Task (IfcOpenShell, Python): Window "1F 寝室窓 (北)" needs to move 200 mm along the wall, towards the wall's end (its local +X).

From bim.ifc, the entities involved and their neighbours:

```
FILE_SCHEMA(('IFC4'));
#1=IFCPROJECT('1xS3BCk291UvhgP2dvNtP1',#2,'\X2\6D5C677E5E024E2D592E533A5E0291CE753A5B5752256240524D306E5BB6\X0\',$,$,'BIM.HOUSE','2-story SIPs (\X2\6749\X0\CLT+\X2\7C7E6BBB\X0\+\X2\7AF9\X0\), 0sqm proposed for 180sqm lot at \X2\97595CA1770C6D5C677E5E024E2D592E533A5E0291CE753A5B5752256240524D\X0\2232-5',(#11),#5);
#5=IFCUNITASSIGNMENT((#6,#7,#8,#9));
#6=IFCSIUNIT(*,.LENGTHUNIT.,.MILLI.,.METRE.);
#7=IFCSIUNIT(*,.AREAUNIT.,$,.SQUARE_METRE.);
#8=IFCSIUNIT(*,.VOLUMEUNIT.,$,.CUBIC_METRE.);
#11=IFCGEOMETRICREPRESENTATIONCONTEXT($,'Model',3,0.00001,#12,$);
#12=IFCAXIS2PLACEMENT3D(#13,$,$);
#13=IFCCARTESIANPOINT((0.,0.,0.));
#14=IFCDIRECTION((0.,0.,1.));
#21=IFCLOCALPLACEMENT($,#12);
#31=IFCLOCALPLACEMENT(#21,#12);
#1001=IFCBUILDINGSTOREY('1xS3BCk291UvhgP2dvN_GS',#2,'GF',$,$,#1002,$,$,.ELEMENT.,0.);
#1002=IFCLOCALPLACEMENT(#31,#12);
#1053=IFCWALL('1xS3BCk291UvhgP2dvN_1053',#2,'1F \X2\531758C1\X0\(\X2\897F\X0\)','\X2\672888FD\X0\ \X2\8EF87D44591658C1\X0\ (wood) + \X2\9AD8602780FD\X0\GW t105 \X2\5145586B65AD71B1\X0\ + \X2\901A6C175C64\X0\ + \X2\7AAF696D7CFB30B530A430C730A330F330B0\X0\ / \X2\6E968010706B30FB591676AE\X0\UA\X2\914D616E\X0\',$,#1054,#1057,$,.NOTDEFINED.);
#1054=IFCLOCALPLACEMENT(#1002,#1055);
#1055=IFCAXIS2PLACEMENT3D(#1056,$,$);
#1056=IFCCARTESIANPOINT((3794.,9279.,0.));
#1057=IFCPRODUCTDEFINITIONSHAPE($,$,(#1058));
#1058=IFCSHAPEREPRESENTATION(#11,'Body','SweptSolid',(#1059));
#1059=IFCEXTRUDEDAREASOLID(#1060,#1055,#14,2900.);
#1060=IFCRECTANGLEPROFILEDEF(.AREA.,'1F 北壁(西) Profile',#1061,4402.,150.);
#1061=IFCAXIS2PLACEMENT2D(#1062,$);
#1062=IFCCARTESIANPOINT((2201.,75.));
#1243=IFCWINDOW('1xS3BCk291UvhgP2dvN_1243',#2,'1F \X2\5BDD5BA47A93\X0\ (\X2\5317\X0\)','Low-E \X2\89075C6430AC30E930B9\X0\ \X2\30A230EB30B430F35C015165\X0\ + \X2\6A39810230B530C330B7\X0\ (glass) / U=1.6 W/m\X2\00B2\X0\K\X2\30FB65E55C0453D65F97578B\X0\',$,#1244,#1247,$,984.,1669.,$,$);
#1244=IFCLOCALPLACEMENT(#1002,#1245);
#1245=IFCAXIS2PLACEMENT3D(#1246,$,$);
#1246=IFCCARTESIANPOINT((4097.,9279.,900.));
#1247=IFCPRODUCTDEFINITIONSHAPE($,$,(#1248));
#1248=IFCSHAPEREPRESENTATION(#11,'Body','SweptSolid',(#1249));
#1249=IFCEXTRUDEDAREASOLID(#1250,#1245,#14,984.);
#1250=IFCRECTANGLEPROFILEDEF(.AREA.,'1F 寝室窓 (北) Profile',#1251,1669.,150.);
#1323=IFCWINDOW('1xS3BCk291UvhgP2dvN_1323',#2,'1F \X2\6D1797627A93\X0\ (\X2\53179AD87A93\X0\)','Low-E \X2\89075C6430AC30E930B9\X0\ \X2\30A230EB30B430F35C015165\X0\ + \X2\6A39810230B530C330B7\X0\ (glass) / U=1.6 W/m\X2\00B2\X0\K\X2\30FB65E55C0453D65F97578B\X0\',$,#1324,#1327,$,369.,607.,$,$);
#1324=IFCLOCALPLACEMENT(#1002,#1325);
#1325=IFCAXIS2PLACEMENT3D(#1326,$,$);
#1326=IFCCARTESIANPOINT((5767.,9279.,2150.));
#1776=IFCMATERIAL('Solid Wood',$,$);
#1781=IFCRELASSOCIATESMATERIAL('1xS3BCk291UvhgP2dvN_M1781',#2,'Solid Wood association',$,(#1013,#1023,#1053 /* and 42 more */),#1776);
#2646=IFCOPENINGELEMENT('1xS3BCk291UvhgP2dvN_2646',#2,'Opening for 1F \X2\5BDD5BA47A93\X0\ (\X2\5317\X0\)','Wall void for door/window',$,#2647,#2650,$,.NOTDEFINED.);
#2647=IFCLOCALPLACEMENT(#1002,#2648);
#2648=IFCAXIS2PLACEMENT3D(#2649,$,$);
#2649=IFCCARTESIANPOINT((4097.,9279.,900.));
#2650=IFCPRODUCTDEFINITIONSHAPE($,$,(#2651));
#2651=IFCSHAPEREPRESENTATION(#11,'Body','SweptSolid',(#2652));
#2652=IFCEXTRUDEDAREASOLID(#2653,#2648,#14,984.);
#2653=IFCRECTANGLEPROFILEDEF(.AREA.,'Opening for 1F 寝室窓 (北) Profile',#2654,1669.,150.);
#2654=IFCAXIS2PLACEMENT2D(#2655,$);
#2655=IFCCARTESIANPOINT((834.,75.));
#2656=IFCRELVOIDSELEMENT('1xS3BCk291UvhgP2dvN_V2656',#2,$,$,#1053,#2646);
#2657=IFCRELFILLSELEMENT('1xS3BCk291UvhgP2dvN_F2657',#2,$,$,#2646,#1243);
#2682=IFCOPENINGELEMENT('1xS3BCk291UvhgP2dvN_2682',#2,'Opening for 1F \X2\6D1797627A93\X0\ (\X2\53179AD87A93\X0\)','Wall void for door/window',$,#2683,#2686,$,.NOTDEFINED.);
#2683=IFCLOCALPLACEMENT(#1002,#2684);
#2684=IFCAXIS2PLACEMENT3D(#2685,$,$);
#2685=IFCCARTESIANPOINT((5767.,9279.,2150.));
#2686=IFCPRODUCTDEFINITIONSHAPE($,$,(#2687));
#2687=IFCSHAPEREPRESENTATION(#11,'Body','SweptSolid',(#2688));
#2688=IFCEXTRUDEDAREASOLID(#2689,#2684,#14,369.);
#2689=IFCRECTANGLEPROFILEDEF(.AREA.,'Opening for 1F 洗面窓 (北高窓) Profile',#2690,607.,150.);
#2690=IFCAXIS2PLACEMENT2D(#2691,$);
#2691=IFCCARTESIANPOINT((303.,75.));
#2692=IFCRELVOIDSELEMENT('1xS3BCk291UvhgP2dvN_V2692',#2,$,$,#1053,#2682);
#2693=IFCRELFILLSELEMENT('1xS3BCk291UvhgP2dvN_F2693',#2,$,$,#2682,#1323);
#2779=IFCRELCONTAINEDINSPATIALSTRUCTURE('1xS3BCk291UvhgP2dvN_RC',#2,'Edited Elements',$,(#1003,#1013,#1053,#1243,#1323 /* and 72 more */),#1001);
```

```python
import ifcopenshell
import ifcopenshell.api.geometry
import ifcopenshell.util.placement
import ifcopenshell.util.unit

model = ifcopenshell.open("bim.ifc")
unit_scale = ifcopenshell.util.unit.calculate_unit_scale(model)

window = model.by_guid("1xS3BCk291UvhgP2dvN_1243")
opening = window.FillsVoids[0].RelatingOpeningElement
wall = opening.VoidsElements[0].RelatingBuildingElement

wall_matrix = ifcopenshell.util.placement.get_local_placement(wall.ObjectPlacement)
shift = wall_matrix[:3, 0] * 0.2 / unit_scale
before = ifcopenshell.util.placement.get_local_placement(window.ObjectPlacement)[:3, 3].copy()

# The window is not placed relative to its opening, so move both.
for product in (opening, window):
    matrix = ifcopenshell.util.placement.get_local_placement(product.ObjectPlacement)
    matrix[:3, 3] += shift
    ifcopenshell.api.geometry.edit_object_placement(model, product=product, matrix=matrix, is_si=False)

after = ifcopenshell.util.placement.get_local_placement(window.ObjectPlacement)[:3, 3]
print("window moved by", (after - before).round(3) + 0.0)

model.write("bim_v2.ifc")
```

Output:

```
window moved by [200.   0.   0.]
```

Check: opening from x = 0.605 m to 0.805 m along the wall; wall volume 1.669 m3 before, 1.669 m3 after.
